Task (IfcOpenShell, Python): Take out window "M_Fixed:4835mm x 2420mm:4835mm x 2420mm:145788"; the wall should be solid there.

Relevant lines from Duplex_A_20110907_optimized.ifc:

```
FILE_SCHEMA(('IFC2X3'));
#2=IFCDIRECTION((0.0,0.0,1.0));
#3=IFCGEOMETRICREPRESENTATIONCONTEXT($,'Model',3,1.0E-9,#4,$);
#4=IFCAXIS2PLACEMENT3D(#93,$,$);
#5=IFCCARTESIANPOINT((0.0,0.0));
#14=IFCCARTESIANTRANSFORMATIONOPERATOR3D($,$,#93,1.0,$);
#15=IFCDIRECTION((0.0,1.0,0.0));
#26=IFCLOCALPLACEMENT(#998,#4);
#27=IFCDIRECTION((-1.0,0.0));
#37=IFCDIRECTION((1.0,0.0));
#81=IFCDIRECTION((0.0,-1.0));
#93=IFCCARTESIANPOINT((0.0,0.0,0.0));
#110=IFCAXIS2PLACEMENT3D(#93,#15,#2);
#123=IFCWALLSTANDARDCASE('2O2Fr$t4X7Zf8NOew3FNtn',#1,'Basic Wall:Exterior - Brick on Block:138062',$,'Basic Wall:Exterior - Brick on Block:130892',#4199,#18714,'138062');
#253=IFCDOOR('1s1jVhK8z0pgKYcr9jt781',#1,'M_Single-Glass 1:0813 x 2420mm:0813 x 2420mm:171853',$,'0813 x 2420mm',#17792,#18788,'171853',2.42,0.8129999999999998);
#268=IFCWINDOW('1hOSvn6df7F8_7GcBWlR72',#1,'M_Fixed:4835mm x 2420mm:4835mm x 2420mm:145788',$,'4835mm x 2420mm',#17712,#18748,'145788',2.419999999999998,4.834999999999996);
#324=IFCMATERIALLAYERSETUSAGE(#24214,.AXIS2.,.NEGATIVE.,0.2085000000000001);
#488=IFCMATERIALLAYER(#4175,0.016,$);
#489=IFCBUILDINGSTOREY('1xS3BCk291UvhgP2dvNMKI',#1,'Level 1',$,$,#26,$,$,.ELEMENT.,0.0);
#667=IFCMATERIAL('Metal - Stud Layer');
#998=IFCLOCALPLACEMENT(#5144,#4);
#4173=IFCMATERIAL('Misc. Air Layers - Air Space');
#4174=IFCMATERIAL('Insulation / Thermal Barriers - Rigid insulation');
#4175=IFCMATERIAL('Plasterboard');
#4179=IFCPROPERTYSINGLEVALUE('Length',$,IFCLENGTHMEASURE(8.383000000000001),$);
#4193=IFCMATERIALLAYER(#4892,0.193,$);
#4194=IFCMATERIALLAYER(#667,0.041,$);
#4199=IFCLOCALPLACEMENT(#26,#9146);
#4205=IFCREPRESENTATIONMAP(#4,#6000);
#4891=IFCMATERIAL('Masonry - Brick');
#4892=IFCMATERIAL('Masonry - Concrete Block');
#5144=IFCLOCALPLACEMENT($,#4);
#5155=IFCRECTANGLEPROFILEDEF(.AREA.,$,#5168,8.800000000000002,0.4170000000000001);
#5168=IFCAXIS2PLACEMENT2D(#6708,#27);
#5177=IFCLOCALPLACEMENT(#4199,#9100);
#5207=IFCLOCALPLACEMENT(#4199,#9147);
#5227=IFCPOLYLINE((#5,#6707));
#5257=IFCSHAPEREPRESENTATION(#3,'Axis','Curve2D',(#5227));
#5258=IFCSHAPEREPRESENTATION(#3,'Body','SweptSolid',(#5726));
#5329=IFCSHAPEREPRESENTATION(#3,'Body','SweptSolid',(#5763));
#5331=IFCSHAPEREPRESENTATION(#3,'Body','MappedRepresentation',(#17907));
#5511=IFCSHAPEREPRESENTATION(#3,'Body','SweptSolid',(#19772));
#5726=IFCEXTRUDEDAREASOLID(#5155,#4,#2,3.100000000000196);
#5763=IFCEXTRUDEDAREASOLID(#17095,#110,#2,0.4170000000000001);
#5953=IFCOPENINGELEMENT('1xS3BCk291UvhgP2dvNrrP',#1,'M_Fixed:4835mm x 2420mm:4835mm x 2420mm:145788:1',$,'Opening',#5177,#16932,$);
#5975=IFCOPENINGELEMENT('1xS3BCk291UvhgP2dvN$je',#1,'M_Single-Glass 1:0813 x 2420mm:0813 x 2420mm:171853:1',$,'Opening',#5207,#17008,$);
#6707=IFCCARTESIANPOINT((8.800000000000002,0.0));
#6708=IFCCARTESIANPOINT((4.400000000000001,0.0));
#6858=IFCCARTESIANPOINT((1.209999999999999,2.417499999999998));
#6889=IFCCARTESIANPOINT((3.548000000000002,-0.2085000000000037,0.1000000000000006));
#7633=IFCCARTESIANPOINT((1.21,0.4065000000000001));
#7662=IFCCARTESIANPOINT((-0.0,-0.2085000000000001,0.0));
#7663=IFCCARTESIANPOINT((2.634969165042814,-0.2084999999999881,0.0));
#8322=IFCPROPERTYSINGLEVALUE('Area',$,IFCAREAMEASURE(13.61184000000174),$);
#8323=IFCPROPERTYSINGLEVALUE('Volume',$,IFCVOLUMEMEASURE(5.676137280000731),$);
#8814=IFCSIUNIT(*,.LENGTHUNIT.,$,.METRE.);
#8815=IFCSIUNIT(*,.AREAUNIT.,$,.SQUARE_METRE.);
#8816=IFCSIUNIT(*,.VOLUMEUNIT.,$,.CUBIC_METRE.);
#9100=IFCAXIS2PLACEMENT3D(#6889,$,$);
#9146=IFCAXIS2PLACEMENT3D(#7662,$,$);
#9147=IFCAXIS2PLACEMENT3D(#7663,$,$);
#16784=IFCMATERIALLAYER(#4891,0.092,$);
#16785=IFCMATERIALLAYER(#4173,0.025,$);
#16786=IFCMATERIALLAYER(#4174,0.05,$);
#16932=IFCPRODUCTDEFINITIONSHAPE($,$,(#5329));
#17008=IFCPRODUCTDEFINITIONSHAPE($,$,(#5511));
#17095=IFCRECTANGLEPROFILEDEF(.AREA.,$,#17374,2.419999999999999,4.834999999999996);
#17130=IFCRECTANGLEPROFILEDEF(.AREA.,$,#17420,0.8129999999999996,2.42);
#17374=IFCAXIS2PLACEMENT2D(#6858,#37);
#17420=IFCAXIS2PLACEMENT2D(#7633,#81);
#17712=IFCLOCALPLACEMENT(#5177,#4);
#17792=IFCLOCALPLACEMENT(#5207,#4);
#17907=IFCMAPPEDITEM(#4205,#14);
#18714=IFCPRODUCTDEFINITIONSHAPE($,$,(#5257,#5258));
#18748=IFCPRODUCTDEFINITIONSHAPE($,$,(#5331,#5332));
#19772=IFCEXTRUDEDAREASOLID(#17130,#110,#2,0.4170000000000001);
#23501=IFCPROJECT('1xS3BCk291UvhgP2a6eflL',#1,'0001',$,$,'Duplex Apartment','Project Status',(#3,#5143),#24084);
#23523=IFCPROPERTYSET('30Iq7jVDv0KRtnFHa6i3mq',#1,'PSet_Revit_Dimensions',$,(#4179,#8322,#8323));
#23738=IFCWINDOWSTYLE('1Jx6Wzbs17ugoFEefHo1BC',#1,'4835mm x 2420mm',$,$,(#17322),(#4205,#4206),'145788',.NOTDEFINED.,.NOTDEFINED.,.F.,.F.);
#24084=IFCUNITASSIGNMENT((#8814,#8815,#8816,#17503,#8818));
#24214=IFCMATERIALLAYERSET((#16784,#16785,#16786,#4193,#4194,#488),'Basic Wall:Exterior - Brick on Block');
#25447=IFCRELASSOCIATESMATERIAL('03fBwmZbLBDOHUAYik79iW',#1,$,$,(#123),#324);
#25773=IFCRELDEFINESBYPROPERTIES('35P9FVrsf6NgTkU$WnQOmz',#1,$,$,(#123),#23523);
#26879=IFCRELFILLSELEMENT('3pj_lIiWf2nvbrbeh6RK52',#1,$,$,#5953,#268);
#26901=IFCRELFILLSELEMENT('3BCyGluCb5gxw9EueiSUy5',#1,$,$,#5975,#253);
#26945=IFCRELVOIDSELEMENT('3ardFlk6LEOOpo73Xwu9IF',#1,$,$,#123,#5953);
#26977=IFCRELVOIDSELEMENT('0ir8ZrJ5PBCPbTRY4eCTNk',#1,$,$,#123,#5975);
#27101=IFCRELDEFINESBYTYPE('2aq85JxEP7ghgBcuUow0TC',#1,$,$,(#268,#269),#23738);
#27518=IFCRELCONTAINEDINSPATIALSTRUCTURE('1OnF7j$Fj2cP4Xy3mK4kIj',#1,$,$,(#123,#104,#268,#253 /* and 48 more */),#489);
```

```python
import ifcopenshell
import ifcopenshell.api.feature
import ifcopenshell.api.pset
import ifcopenshell.api.root
import ifcopenshell.geom
import ifcopenshell.util.element
import ifcopenshell.util.shape
import ifcopenshell.util.unit

model = ifcopenshell.open("Duplex_A_20110907_optimized.ifc")
area_scale = ifcopenshell.util.unit.calculate_unit_scale(model, "AREAUNIT")
volume_scale = ifcopenshell.util.unit.calculate_unit_scale(model, "VOLUMEUNIT")
settings = ifcopenshell.geom.settings()


def volume(element):
    """Net volume in cubic metres, openings subtracted."""
    shape = ifcopenshell.geom.create_shape(settings, element)
    return ifcopenshell.util.shape.get_volume(shape.geometry)


window = model.by_guid("1hOSvn6df7F8_7GcBWlR72")
opening = window.FillsVoids[0].RelatingOpeningElement
wall = opening.VoidsElements[0].RelatingBuildingElement
before = volume(wall)

ifcopenshell.api.root.remove_product(model, product=window)
ifcopenshell.api.feature.remove_feature(model, feature=opening)

after = volume(wall)
thickness = 0.417  # wall thickness in metres

# Update the wall's stored quantities.
pset = model.by_id(ifcopenshell.util.element.get_pset(wall, "PSet_Revit_Dimensions", should_inherit=False)["id"])
ifcopenshell.api.pset.edit_pset(model, pset=pset, properties={
    "Area": model.create_entity("IfcAreaMeasure", after / thickness / area_scale),
    "Volume": model.create_entity("IfcVolumeMeasure", after / volume_scale),
})

print(f"wall volume {before:.3f} -> {after:.3f} m3")

model.write("Duplex_A_20110907_optimized_v2.ifc")
```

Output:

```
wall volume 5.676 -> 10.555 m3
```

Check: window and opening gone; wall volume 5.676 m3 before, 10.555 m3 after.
